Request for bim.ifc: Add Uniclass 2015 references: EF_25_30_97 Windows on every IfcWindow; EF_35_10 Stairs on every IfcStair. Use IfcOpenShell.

First a look at what the model holds.

```python
import ifcopenshell

model = ifcopenshell.open("bim.ifc")
print(model.schema)
print("classifications:", [c.Name for c in model.by_type("IfcClassification")])
for ifc_class in ("IfcDoor", "IfcRoof", "IfcStair", "IfcWall", "IfcWindow"):
    print(ifc_class, len(model.by_type(ifc_class)))
```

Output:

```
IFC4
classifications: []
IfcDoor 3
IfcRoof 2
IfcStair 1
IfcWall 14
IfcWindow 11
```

```python
import ifcopenshell
import ifcopenshell.api.classification

model = ifcopenshell.open("bim.ifc")

system = ifcopenshell.api.classification.add_classification(model, classification="Uniclass 2015")

codes = {
    "IfcWindow": ("EF_25_30_97", "Windows"),
    "IfcStair": ("EF_35_10", "Stairs"),
}
for ifc_class, (code, name) in codes.items():
    products = model.by_type(ifc_class)
    ifcopenshell.api.classification.add_reference(
        model, products=products, classification=system, identification=code, name=name
    )
    print(code, len(products))

model.write("bim_updated.ifc")
```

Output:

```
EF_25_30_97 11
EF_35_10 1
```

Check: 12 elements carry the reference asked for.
